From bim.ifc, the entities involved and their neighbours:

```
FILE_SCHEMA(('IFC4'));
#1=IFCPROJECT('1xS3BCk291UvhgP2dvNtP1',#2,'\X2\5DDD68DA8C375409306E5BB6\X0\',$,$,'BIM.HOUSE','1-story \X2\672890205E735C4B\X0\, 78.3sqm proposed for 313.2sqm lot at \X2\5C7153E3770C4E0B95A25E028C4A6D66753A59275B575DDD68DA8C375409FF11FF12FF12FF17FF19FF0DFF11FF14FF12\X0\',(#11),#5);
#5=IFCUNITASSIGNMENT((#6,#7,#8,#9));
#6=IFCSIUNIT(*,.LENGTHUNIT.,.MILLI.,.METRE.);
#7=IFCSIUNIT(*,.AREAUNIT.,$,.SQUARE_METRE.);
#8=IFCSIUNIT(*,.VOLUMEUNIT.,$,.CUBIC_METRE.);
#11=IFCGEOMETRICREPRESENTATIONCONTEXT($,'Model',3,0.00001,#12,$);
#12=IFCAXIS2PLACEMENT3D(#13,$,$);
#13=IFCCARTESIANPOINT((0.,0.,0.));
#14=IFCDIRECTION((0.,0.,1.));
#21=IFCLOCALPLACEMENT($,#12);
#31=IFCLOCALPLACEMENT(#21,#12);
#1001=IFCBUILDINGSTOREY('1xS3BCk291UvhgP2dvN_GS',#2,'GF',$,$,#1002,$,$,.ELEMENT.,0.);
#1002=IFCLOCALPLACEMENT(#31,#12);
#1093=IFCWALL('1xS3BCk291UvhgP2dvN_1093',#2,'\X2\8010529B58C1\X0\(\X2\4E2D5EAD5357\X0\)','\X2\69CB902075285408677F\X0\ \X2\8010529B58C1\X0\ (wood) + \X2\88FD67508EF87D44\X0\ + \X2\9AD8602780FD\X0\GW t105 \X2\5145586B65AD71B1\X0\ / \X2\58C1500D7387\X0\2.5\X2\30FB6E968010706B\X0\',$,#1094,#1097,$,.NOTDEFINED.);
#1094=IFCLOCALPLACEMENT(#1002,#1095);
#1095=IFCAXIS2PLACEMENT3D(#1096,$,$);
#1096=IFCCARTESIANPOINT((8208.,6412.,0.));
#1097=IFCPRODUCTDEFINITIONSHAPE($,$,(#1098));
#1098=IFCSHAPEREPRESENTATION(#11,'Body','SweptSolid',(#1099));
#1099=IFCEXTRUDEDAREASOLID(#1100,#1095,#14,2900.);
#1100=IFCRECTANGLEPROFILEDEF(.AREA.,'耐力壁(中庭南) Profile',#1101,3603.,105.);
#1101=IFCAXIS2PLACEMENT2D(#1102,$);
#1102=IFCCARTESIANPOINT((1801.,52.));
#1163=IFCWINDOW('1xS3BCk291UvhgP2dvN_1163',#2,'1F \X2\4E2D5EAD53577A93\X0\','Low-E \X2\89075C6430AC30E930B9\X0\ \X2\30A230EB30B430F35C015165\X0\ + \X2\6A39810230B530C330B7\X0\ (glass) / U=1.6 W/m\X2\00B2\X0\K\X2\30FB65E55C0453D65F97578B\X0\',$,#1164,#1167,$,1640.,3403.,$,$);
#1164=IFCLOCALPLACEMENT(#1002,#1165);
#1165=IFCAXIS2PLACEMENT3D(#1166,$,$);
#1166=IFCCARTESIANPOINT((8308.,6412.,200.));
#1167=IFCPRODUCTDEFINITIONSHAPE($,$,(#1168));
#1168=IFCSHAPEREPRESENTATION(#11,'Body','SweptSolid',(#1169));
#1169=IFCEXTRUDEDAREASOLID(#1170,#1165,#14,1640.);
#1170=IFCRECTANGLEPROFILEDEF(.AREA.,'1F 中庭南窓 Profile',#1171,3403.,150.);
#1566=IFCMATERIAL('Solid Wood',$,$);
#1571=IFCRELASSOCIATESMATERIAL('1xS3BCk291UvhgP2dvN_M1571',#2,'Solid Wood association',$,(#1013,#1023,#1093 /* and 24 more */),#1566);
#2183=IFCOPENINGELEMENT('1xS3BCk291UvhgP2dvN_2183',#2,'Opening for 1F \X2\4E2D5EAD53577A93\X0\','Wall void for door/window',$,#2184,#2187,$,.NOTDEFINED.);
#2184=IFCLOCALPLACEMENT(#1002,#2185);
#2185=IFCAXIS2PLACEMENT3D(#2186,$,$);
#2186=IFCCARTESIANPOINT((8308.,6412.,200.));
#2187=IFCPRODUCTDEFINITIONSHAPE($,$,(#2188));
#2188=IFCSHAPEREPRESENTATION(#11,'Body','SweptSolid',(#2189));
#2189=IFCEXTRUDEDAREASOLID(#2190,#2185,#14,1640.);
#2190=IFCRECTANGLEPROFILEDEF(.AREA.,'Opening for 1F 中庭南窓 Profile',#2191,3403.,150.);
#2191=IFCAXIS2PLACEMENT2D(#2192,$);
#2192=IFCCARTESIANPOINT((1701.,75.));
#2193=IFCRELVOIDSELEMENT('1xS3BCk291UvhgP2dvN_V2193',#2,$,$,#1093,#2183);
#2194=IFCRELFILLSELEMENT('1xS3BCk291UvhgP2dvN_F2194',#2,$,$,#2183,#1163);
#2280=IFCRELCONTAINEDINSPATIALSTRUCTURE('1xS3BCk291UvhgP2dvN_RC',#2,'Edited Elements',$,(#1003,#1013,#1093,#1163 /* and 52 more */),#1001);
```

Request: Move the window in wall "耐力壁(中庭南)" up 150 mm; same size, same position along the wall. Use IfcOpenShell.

```python
import numpy as np
import ifcopenshell
import ifcopenshell.api.geometry
import ifcopenshell.util.placement
import ifcopenshell.util.unit

model = ifcopenshell.open("bim.ifc")
unit_scale = ifcopenshell.util.unit.calculate_unit_scale(model)

window = model.by_guid("1xS3BCk291UvhgP2dvN_1163")
opening = window.FillsVoids[0].RelatingOpeningElement
dz = 0.15 / unit_scale

shift = np.array([0.0, 0.0, dz])
# The window is not placed relative to its opening, so move both.
for product in (opening, window):
    matrix = ifcopenshell.util.placement.get_local_placement(product.ObjectPlacement)
    matrix[:3, 3] += shift
    ifcopenshell.api.geometry.edit_object_placement(model, product=product, matrix=matrix, is_si=False)

print(f"moved by {dz * unit_scale:+.3f} m")

model.write("bim_rev.ifc")
```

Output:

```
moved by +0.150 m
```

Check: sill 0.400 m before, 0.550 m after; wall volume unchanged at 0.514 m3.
